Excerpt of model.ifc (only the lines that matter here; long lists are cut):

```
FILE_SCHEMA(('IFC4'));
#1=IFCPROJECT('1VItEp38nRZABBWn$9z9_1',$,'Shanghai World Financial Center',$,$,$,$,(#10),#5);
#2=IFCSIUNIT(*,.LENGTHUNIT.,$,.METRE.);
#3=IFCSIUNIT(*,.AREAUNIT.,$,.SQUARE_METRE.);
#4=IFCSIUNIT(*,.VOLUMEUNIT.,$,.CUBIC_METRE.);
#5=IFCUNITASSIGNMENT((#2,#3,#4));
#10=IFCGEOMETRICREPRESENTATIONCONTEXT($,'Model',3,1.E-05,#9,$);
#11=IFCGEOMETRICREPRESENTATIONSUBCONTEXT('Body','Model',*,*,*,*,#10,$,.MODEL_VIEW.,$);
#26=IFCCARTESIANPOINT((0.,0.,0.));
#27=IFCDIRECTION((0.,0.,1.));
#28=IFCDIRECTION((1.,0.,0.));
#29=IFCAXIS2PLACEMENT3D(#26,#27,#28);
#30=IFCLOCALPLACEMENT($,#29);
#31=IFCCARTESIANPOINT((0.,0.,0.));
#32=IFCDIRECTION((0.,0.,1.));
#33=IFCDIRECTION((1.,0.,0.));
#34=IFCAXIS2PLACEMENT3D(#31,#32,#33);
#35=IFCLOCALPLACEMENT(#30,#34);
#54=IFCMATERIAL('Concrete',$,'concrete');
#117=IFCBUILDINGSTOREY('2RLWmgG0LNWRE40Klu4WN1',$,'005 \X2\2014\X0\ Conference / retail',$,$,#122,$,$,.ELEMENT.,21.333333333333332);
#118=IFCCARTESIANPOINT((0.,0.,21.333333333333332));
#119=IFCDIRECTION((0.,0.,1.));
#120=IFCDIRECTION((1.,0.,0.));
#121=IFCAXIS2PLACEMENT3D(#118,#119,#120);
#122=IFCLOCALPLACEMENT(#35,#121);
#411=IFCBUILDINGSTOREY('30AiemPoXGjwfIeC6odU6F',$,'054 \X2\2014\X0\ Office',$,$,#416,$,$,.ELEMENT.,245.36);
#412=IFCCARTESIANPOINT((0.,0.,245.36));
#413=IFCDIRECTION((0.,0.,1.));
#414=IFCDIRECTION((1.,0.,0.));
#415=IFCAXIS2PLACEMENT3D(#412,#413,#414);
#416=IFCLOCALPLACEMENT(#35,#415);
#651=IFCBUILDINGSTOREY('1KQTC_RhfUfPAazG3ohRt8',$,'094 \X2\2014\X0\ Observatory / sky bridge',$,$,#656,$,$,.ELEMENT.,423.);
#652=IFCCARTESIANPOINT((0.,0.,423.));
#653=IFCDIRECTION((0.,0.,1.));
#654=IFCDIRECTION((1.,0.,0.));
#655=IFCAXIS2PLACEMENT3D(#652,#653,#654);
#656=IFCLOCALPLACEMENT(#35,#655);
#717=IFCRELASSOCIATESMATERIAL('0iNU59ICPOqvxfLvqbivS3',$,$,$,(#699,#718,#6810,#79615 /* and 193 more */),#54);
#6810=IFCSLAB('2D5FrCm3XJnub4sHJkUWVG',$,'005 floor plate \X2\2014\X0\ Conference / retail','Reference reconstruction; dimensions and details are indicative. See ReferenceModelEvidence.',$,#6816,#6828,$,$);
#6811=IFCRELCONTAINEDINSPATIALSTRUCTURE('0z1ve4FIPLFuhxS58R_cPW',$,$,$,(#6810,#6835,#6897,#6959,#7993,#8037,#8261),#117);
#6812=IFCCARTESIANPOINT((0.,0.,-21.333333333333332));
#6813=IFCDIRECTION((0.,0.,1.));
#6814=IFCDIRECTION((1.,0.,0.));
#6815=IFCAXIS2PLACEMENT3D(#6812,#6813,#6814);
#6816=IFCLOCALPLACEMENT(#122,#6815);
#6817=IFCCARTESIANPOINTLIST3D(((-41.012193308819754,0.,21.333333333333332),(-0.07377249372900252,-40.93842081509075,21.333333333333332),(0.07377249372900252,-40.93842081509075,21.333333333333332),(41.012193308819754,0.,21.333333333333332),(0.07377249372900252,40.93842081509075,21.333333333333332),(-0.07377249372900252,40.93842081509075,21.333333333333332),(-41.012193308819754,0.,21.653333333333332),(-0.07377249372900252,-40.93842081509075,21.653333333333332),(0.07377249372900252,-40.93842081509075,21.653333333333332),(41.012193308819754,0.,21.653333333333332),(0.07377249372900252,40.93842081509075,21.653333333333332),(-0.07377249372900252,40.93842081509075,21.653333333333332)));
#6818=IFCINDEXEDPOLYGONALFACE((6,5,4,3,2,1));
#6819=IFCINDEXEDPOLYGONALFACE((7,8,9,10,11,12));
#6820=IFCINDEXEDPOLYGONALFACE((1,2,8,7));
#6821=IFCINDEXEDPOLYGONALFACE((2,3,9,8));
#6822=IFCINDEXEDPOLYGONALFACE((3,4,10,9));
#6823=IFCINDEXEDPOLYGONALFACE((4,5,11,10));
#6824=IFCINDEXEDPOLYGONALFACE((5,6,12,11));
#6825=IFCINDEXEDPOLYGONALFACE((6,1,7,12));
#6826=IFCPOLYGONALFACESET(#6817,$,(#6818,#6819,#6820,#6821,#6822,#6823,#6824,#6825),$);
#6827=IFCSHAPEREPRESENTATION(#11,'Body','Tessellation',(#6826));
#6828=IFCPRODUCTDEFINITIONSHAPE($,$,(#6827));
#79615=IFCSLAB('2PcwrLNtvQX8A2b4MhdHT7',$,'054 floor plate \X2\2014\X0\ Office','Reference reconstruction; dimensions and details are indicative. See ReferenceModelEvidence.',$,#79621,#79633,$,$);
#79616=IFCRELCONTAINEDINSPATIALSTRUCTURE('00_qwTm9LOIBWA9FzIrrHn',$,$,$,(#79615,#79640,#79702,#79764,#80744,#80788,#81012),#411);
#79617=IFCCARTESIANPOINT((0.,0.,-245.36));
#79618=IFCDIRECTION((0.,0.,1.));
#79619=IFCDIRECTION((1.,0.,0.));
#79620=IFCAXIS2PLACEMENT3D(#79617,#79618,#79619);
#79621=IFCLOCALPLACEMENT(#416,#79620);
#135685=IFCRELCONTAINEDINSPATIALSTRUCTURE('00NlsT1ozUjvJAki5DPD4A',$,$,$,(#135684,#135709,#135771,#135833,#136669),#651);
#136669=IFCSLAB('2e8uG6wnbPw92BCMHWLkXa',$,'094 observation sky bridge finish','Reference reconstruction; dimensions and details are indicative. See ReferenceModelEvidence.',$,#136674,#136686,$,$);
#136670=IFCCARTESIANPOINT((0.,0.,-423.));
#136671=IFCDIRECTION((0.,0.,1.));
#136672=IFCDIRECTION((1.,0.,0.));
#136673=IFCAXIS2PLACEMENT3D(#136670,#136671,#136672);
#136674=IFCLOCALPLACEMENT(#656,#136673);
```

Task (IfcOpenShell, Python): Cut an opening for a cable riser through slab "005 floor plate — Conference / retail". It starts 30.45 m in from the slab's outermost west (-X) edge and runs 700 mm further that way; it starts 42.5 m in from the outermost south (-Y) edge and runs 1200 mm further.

```python
import numpy as np
import ifcopenshell
import ifcopenshell.api.feature
import ifcopenshell.api.geometry
import ifcopenshell.api.root
import ifcopenshell.geom
import ifcopenshell.util.placement
import ifcopenshell.util.representation
import ifcopenshell.util.shape
import ifcopenshell.util.unit

model = ifcopenshell.open("model.ifc")
unit_scale = ifcopenshell.util.unit.calculate_unit_scale(model)
settings = ifcopenshell.geom.settings()


def volume(element):
    """Net volume in cubic metres, openings subtracted."""
    shape = ifcopenshell.geom.create_shape(settings, element)
    return ifcopenshell.util.shape.get_volume(shape.geometry)


slab = model.by_guid("2D5FrCm3XJnub4sHJkUWVG")
before = volume(slab)

# Extent in the slab's own axes, in metres. The edges named are its -X and -Y sides.
slab_shape = ifcopenshell.geom.create_shape(settings, slab)
vertices = ifcopenshell.util.shape.get_vertices(slab_shape.geometry)
x_min, y_min, bottom = vertices.min(axis=0)
top = vertices[:, 2].max()

opening = ifcopenshell.api.root.create_entity(model, ifc_class="IfcOpeningElement", name="Cable riser opening", predefined_type="OPENING")
context = ifcopenshell.util.representation.get_context(model, "Model", "Body", "MODEL_VIEW")
width, depth = 0.7, 1.2
outline = [(0.0, 0.0), (width, 0.0), (width, depth), (0.0, depth), (0.0, 0.0)]
# Overshoot both faces by 50 mm so the cut is clean.
shape = ifcopenshell.api.geometry.add_slab_representation(
    model, context=context, depth=top - bottom + 0.1, polyline=outline
)
ifcopenshell.api.geometry.assign_representation(model, product=opening, representation=shape)

matrix = ifcopenshell.util.placement.get_local_placement(slab.ObjectPlacement)
matrix[:, 3] = matrix @ np.append(np.array([x_min + 30.45, y_min + 42.5, bottom - 0.05]) / unit_scale, 1.0)
ifcopenshell.api.geometry.edit_object_placement(model, product=opening, matrix=matrix, is_si=False)
ifcopenshell.api.feature.add_feature(model, feature=opening, element=slab)

after = volume(slab)

print(f"slab volume {before:.3f} -> {after:.3f} m3")

model.write("model_rev.ifc")
```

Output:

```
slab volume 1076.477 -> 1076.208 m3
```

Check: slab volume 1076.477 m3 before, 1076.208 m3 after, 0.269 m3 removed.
